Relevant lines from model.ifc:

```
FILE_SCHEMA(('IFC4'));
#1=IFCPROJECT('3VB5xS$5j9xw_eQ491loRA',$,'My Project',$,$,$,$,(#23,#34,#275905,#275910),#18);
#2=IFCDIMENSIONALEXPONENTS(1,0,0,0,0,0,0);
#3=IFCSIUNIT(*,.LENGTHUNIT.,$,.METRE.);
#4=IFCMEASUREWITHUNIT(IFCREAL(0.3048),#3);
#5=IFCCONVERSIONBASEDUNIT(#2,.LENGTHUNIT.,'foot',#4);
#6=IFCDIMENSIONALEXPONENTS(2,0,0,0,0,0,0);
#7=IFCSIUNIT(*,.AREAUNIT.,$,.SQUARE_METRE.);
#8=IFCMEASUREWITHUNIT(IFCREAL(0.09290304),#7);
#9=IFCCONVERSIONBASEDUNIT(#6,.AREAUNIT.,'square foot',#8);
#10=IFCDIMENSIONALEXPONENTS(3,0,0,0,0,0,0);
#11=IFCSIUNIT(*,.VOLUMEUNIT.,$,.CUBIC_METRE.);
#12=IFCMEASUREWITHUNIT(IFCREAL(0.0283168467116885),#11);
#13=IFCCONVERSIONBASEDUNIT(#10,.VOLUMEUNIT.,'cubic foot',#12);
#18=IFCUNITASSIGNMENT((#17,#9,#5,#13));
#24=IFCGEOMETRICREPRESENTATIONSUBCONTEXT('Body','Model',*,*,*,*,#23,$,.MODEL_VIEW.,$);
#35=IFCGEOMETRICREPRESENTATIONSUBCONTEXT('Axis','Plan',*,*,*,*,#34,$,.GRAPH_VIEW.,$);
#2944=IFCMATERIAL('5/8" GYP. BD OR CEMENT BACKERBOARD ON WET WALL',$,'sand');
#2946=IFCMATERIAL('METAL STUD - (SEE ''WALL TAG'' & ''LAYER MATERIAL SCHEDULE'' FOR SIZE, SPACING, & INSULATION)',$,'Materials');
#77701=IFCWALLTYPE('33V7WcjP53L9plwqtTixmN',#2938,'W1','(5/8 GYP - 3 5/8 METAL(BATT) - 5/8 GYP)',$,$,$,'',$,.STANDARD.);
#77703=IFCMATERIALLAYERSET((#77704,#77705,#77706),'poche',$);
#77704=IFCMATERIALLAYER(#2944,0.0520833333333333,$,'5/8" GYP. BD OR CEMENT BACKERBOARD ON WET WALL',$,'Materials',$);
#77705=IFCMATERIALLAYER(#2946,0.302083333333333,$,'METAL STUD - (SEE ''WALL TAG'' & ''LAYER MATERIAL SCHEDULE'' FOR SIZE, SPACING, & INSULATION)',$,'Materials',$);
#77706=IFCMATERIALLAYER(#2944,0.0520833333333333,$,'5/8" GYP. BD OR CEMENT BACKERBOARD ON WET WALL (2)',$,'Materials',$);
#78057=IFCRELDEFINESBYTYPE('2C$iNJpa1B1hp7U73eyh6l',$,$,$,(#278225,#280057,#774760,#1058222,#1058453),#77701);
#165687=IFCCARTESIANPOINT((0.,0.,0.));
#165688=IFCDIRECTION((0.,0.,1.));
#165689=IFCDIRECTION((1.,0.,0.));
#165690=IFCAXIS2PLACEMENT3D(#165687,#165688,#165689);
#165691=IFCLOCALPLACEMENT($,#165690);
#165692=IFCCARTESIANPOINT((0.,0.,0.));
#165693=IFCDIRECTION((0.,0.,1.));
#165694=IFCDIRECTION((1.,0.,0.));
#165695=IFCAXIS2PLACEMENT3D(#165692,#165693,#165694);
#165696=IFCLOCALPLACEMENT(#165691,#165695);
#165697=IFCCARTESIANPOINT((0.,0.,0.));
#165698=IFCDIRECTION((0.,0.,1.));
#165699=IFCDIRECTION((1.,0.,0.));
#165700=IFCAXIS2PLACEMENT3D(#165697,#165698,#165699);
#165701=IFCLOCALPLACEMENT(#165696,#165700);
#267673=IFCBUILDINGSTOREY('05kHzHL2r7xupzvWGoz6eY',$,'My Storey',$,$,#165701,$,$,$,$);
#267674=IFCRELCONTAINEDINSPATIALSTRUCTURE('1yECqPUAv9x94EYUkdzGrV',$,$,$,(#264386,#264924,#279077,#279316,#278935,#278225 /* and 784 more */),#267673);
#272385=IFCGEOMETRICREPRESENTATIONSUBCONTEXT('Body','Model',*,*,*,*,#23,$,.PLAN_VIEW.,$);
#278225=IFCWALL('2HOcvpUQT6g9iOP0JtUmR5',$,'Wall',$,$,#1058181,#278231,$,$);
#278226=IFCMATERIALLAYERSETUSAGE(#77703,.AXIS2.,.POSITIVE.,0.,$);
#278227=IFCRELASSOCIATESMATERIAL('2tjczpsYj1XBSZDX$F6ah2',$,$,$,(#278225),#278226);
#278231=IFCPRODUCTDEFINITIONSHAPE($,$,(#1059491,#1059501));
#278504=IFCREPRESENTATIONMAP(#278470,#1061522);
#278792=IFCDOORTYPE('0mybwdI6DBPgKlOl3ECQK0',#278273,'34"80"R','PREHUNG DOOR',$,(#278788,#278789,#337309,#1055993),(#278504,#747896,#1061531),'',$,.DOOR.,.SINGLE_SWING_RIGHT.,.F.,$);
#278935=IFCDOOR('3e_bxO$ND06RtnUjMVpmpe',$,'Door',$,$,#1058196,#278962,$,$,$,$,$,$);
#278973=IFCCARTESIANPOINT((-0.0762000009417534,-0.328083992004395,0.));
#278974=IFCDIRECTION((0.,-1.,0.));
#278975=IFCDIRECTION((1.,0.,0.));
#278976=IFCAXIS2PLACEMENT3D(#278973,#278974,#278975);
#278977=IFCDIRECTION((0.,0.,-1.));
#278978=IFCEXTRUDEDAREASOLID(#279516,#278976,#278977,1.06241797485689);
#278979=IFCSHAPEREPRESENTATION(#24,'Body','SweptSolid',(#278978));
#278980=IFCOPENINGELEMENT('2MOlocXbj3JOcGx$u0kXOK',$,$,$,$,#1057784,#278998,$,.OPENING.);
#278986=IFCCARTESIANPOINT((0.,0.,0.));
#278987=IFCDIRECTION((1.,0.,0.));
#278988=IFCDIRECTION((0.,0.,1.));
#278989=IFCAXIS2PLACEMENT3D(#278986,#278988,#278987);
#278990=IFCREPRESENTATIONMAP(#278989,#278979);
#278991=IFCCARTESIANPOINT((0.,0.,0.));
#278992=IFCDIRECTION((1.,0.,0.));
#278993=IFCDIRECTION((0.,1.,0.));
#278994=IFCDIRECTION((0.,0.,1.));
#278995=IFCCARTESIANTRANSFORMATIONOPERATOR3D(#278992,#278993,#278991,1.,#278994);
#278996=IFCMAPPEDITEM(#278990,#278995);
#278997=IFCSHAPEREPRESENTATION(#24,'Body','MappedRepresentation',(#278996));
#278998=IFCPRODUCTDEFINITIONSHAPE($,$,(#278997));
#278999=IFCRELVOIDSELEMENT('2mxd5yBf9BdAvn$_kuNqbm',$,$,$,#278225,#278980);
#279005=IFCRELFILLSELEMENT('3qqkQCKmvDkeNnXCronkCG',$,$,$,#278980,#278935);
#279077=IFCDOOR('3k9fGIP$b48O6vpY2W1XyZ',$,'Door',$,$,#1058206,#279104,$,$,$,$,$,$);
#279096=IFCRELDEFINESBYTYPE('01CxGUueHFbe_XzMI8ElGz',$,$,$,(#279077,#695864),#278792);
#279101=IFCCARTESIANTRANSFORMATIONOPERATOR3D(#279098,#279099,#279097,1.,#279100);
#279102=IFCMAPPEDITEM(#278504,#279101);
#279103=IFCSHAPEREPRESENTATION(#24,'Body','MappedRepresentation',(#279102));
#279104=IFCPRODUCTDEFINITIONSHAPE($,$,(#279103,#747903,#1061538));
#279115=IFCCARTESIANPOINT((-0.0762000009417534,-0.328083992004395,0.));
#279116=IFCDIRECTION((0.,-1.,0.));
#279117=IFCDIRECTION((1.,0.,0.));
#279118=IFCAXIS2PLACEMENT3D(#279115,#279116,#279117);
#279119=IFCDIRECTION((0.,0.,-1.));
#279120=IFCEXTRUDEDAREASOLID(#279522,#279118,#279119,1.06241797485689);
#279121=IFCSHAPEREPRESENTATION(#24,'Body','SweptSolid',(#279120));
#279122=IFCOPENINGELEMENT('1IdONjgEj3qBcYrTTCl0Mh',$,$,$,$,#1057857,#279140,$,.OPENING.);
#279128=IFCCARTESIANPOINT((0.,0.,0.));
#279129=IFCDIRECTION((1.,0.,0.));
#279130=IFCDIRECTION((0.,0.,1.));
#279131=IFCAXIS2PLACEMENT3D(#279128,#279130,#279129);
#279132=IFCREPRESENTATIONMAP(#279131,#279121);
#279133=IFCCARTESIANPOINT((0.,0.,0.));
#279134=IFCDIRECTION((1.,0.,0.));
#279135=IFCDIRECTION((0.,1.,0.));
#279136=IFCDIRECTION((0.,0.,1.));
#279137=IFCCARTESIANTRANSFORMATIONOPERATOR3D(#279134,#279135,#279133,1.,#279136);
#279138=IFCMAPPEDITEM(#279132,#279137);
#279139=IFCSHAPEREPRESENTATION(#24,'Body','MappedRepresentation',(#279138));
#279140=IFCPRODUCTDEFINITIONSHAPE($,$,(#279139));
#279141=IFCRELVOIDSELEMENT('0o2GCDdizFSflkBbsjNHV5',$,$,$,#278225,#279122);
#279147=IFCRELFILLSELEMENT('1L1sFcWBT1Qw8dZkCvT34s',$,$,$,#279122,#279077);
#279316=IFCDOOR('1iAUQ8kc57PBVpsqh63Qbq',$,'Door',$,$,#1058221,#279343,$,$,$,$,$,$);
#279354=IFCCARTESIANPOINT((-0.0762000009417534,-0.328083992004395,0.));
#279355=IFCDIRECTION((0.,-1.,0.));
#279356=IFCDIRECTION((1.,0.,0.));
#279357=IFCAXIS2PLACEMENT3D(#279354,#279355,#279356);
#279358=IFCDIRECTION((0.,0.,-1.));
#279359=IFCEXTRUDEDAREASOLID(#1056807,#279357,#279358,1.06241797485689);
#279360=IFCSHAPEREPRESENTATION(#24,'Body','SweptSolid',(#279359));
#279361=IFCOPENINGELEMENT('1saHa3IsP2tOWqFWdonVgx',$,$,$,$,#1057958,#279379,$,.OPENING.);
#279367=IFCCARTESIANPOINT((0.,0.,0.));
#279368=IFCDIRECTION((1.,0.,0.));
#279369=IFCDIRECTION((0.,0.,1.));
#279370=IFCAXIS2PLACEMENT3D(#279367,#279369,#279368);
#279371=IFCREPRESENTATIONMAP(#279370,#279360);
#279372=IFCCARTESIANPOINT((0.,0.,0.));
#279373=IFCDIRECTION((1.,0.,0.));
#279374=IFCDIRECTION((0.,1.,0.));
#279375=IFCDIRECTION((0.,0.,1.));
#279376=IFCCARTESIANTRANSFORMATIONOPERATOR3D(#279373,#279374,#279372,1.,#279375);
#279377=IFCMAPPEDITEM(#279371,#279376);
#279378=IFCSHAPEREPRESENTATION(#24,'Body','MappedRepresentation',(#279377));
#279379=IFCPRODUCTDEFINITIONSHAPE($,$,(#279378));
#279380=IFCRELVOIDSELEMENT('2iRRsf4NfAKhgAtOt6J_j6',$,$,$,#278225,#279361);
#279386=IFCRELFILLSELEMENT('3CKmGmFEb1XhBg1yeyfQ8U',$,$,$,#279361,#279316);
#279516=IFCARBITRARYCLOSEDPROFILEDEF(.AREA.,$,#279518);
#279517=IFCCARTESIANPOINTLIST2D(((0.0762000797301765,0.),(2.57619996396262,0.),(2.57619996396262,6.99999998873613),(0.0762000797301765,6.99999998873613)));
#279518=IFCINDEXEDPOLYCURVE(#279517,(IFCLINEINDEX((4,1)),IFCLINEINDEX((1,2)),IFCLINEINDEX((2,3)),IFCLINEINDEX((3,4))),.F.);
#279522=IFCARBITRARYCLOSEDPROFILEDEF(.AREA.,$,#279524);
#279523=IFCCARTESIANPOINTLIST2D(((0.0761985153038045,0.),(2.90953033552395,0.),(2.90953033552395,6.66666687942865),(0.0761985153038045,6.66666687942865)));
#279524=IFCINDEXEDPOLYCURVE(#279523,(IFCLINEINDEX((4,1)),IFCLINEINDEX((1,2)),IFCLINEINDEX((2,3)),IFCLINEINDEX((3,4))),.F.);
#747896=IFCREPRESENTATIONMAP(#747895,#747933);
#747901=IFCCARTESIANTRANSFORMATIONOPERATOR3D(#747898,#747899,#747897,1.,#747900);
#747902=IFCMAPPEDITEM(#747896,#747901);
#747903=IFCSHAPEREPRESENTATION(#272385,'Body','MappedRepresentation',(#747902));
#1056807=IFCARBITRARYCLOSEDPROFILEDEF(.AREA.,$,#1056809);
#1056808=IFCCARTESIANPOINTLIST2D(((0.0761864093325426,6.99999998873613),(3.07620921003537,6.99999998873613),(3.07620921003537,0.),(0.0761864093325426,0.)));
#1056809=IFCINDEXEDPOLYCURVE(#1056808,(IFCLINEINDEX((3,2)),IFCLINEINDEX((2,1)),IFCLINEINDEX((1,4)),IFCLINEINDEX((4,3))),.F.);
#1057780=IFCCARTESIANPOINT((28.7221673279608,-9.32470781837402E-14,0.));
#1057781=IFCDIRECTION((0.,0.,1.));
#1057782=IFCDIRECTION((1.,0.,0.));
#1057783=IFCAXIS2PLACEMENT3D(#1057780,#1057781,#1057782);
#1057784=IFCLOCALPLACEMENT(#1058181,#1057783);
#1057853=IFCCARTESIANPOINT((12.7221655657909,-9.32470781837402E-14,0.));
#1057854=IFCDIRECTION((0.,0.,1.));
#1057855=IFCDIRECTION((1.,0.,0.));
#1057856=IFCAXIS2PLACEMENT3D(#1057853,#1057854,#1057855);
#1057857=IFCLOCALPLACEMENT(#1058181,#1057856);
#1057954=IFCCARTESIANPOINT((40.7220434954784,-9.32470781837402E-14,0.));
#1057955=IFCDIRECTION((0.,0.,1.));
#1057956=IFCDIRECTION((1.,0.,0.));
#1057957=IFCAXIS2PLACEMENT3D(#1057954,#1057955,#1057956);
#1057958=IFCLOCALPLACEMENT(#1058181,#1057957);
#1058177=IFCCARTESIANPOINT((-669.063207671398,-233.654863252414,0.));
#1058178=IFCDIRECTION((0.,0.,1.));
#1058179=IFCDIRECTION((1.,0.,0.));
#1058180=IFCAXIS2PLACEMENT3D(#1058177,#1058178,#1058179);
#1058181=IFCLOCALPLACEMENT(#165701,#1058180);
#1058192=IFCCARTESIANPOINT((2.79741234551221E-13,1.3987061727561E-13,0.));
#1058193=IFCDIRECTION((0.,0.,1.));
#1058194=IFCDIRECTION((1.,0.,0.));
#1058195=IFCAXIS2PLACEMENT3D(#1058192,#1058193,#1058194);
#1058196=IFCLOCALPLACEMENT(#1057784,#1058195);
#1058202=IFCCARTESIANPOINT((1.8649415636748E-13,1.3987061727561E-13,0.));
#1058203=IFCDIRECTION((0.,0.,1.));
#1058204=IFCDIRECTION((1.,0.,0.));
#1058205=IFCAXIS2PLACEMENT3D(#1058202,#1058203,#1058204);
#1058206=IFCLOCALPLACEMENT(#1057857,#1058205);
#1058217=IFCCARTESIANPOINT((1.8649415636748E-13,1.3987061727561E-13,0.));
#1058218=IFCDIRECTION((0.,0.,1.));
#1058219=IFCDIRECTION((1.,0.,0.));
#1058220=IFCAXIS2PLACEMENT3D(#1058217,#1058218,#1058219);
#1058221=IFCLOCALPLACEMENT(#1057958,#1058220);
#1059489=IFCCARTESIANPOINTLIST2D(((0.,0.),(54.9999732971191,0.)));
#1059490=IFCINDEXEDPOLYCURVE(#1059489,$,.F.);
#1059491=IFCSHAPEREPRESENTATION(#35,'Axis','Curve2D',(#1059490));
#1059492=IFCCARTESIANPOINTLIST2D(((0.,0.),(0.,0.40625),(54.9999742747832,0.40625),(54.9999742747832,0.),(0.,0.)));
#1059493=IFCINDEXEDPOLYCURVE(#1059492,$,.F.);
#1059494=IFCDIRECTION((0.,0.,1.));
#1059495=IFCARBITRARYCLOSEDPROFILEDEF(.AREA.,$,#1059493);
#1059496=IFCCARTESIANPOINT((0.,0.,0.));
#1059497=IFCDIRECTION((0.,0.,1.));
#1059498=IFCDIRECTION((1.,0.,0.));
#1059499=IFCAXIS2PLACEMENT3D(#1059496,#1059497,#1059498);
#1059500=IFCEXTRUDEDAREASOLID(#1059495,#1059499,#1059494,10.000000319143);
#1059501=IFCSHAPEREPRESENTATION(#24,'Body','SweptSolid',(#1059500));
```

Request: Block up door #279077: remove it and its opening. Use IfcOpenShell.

```python
import ifcopenshell
import ifcopenshell.api.feature
import ifcopenshell.api.root
import ifcopenshell.geom
import ifcopenshell.util.shape

model = ifcopenshell.open("model.ifc")
settings = ifcopenshell.geom.settings()


def volume(element):
    """Net volume in cubic metres, openings subtracted."""
    shape = ifcopenshell.geom.create_shape(settings, element)
    return ifcopenshell.util.shape.get_volume(shape.geometry)


door = model.by_id(279077)
opening = door.FillsVoids[0].RelatingOpeningElement
wall = opening.VoidsElements[0].RelatingBuildingElement
before = volume(wall)

ifcopenshell.api.root.remove_product(model, product=door)
ifcopenshell.api.feature.remove_feature(model, feature=opening)

after = volume(wall)

print(f"wall volume {before:.3f} -> {after:.3f} m3")

model.write("model-out.ifc")
```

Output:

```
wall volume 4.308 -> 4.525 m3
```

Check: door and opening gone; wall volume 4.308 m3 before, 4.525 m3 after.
